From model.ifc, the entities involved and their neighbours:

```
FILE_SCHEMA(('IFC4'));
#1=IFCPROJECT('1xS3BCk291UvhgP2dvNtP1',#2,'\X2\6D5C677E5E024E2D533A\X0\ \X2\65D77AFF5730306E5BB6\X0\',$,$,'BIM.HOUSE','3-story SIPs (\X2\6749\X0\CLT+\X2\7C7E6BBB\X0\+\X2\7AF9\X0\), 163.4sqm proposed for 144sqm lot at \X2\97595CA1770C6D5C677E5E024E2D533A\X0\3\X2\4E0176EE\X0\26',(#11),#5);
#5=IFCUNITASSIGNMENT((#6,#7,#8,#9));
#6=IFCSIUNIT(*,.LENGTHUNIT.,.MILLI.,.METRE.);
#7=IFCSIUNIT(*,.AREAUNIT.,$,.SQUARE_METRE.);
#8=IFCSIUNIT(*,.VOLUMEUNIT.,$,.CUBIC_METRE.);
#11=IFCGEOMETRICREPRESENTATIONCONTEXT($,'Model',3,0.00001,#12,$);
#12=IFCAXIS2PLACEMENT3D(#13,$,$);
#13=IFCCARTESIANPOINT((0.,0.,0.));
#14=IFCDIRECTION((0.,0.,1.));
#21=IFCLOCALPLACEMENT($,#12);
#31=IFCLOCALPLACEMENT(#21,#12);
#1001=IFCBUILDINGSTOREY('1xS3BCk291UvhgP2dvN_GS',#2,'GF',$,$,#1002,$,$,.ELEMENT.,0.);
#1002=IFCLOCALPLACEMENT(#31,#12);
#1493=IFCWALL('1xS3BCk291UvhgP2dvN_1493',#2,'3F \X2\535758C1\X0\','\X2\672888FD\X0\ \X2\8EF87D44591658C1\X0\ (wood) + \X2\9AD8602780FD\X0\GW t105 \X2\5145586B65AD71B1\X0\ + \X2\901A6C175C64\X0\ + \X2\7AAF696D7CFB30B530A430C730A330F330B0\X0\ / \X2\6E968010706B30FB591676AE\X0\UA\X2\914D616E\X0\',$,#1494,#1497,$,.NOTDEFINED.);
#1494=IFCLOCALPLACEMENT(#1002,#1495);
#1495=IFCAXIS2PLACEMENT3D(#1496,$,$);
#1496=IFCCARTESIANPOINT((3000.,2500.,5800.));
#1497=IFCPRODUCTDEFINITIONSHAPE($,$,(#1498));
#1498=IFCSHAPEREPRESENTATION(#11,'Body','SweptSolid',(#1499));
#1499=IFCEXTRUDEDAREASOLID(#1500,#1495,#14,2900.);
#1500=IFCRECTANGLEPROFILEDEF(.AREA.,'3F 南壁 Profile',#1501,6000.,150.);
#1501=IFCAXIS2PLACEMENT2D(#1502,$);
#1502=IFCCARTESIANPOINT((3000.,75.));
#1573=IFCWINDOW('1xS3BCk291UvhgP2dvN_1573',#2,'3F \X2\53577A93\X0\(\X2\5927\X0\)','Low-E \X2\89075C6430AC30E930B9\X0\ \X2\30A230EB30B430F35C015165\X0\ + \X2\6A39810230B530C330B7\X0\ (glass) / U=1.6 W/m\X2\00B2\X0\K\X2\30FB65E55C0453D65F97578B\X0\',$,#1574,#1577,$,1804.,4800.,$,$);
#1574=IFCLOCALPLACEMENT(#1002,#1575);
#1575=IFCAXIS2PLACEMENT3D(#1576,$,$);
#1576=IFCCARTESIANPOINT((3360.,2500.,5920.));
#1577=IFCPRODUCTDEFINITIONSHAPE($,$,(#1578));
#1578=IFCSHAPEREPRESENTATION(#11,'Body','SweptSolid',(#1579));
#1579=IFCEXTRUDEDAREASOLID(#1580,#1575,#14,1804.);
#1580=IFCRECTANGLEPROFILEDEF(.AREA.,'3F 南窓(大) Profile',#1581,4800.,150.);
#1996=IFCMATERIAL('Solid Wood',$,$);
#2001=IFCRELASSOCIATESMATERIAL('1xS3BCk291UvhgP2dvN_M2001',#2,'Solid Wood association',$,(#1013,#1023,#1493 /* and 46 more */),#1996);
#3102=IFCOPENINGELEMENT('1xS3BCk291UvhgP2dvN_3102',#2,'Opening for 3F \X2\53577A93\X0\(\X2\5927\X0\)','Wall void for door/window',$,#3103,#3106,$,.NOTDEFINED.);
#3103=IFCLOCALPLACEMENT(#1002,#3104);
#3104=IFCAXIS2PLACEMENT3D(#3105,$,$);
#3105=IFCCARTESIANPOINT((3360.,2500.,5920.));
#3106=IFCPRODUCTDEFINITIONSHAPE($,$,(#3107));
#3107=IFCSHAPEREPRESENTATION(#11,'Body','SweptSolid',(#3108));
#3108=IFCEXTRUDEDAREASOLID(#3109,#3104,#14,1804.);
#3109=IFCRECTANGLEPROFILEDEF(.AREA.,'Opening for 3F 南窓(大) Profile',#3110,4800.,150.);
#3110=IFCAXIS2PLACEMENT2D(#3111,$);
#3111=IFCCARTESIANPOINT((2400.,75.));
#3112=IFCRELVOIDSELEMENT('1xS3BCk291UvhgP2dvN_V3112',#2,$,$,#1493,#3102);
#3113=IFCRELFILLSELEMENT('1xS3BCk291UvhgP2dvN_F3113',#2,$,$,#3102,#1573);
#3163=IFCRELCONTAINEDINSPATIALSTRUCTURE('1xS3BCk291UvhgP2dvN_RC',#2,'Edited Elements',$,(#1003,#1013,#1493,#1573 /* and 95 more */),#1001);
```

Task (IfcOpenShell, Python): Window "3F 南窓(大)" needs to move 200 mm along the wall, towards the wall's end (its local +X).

```python
import ifcopenshell
import ifcopenshell.api.geometry
import ifcopenshell.util.placement
import ifcopenshell.util.unit

model = ifcopenshell.open("model.ifc")
unit_scale = ifcopenshell.util.unit.calculate_unit_scale(model)

window = model.by_guid("1xS3BCk291UvhgP2dvN_1573")
opening = window.FillsVoids[0].RelatingOpeningElement
wall = opening.VoidsElements[0].RelatingBuildingElement

wall_matrix = ifcopenshell.util.placement.get_local_placement(wall.ObjectPlacement)
shift = wall_matrix[:3, 0] * 0.2 / unit_scale
before = ifcopenshell.util.placement.get_local_placement(window.ObjectPlacement)[:3, 3].copy()

# The window is not placed relative to its opening, so move both.
for product in (opening, window):
    matrix = ifcopenshell.util.placement.get_local_placement(product.ObjectPlacement)
    matrix[:3, 3] += shift
    ifcopenshell.api.geometry.edit_object_placement(model, product=product, matrix=matrix, is_si=False)

after = ifcopenshell.util.placement.get_local_placement(window.ObjectPlacement)[:3, 3]
print("window moved by", (after - before).round(3) + 0.0)

model.write("model_updated.ifc")
```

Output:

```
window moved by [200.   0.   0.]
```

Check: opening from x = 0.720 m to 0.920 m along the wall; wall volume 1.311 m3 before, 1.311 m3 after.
